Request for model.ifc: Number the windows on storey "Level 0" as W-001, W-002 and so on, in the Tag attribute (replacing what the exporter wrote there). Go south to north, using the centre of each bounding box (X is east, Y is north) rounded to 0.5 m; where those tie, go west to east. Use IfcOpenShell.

First a look at what the model holds.

```python
import ifcopenshell
import ifcopenshell.util.element
import ifcopenshell.util.placement

model = ifcopenshell.open("model.ifc")
print(model.schema)
storey = next(s for s in model.by_type("IfcBuildingStorey") if s.Name == "Level 0")
windows = [e for e in ifcopenshell.util.element.get_decomposition(storey) if e.is_a("IfcWindow")]
for e in sorted(windows, key=lambda e: e.id()):
    origin = ifcopenshell.util.placement.get_local_placement(e.ObjectPlacement)[:3, 3]
    print(e.id(), e.Tag, e.Name, origin.round(2) + 0.0, sep=" | ")
```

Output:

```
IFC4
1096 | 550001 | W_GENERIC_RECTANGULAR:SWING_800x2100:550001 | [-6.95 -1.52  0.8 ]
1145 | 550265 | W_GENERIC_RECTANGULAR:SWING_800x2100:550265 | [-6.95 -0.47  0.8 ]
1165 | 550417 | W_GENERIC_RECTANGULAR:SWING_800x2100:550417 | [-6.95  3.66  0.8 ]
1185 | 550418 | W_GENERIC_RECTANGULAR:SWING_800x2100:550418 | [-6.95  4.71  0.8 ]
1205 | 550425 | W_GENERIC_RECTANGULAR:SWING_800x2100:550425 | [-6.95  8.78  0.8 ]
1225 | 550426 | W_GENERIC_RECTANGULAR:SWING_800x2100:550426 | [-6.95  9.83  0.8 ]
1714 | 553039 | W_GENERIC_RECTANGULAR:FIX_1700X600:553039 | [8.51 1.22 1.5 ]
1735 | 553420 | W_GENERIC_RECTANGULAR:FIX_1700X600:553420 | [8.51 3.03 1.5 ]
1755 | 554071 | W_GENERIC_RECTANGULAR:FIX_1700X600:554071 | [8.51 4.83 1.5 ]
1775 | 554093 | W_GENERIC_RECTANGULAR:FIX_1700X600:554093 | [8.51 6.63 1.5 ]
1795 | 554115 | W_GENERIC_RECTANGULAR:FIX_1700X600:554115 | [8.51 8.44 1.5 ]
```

```python
import ifcopenshell
import ifcopenshell.geom
import ifcopenshell.util.element
import ifcopenshell.util.shape

model = ifcopenshell.open("model.ifc")
settings = ifcopenshell.geom.settings()
settings.set("use-world-coords", True)


def centre(element):
    shape = ifcopenshell.geom.create_shape(settings, element)
    return ifcopenshell.util.shape.get_bbox_centroid(shape.geometry)


storey = next(s for s in model.by_type("IfcBuildingStorey") if s.Name == "Level 0")
windows = [e for e in ifcopenshell.util.element.get_decomposition(storey) if e.is_a("IfcWindow")]

# Insertion points can sit at a corner or the storey origin, so sort by the geometry (in metres).
centres = {e: centre(e) for e in windows}
windows.sort(key=lambda e: (round(centres[e][1] / 0.5), centres[e][0]))

for i, e in enumerate(windows, start=1):
    number = f"W-0{i:02d}"
    e.Tag = number
    print(e.id(), number)

model.write("model_updated.ifc")
```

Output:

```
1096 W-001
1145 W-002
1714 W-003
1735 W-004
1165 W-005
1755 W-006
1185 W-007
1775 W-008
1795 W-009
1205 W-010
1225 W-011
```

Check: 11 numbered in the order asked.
